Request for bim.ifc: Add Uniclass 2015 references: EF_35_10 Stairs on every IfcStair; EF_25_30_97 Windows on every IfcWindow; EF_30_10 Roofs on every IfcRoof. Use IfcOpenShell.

First a look at what the model holds.

```python
import ifcopenshell

model = ifcopenshell.open("bim.ifc")
print(model.schema)
print("classifications:", [c.Name for c in model.by_type("IfcClassification")])
for ifc_class in ("IfcDoor", "IfcRoof", "IfcStair", "IfcWall", "IfcWindow"):
    print(ifc_class, len(model.by_type(ifc_class)))
```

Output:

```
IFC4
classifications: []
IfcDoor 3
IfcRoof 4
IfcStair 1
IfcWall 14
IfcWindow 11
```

```python
import ifcopenshell
import ifcopenshell.api.classification

model = ifcopenshell.open("bim.ifc")

system = ifcopenshell.api.classification.add_classification(model, classification="Uniclass 2015")

codes = {
    "IfcStair": ("EF_35_10", "Stairs"),
    "IfcWindow": ("EF_25_30_97", "Windows"),
    "IfcRoof": ("EF_30_10", "Roofs"),
}
for ifc_class, (code, name) in codes.items():
    products = model.by_type(ifc_class)
    ifcopenshell.api.classification.add_reference(
        model, products=products, classification=system, identification=code, name=name
    )
    print(code, len(products))

model.write("bim_edited.ifc")
```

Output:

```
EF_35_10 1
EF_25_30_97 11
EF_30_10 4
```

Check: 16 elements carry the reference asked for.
